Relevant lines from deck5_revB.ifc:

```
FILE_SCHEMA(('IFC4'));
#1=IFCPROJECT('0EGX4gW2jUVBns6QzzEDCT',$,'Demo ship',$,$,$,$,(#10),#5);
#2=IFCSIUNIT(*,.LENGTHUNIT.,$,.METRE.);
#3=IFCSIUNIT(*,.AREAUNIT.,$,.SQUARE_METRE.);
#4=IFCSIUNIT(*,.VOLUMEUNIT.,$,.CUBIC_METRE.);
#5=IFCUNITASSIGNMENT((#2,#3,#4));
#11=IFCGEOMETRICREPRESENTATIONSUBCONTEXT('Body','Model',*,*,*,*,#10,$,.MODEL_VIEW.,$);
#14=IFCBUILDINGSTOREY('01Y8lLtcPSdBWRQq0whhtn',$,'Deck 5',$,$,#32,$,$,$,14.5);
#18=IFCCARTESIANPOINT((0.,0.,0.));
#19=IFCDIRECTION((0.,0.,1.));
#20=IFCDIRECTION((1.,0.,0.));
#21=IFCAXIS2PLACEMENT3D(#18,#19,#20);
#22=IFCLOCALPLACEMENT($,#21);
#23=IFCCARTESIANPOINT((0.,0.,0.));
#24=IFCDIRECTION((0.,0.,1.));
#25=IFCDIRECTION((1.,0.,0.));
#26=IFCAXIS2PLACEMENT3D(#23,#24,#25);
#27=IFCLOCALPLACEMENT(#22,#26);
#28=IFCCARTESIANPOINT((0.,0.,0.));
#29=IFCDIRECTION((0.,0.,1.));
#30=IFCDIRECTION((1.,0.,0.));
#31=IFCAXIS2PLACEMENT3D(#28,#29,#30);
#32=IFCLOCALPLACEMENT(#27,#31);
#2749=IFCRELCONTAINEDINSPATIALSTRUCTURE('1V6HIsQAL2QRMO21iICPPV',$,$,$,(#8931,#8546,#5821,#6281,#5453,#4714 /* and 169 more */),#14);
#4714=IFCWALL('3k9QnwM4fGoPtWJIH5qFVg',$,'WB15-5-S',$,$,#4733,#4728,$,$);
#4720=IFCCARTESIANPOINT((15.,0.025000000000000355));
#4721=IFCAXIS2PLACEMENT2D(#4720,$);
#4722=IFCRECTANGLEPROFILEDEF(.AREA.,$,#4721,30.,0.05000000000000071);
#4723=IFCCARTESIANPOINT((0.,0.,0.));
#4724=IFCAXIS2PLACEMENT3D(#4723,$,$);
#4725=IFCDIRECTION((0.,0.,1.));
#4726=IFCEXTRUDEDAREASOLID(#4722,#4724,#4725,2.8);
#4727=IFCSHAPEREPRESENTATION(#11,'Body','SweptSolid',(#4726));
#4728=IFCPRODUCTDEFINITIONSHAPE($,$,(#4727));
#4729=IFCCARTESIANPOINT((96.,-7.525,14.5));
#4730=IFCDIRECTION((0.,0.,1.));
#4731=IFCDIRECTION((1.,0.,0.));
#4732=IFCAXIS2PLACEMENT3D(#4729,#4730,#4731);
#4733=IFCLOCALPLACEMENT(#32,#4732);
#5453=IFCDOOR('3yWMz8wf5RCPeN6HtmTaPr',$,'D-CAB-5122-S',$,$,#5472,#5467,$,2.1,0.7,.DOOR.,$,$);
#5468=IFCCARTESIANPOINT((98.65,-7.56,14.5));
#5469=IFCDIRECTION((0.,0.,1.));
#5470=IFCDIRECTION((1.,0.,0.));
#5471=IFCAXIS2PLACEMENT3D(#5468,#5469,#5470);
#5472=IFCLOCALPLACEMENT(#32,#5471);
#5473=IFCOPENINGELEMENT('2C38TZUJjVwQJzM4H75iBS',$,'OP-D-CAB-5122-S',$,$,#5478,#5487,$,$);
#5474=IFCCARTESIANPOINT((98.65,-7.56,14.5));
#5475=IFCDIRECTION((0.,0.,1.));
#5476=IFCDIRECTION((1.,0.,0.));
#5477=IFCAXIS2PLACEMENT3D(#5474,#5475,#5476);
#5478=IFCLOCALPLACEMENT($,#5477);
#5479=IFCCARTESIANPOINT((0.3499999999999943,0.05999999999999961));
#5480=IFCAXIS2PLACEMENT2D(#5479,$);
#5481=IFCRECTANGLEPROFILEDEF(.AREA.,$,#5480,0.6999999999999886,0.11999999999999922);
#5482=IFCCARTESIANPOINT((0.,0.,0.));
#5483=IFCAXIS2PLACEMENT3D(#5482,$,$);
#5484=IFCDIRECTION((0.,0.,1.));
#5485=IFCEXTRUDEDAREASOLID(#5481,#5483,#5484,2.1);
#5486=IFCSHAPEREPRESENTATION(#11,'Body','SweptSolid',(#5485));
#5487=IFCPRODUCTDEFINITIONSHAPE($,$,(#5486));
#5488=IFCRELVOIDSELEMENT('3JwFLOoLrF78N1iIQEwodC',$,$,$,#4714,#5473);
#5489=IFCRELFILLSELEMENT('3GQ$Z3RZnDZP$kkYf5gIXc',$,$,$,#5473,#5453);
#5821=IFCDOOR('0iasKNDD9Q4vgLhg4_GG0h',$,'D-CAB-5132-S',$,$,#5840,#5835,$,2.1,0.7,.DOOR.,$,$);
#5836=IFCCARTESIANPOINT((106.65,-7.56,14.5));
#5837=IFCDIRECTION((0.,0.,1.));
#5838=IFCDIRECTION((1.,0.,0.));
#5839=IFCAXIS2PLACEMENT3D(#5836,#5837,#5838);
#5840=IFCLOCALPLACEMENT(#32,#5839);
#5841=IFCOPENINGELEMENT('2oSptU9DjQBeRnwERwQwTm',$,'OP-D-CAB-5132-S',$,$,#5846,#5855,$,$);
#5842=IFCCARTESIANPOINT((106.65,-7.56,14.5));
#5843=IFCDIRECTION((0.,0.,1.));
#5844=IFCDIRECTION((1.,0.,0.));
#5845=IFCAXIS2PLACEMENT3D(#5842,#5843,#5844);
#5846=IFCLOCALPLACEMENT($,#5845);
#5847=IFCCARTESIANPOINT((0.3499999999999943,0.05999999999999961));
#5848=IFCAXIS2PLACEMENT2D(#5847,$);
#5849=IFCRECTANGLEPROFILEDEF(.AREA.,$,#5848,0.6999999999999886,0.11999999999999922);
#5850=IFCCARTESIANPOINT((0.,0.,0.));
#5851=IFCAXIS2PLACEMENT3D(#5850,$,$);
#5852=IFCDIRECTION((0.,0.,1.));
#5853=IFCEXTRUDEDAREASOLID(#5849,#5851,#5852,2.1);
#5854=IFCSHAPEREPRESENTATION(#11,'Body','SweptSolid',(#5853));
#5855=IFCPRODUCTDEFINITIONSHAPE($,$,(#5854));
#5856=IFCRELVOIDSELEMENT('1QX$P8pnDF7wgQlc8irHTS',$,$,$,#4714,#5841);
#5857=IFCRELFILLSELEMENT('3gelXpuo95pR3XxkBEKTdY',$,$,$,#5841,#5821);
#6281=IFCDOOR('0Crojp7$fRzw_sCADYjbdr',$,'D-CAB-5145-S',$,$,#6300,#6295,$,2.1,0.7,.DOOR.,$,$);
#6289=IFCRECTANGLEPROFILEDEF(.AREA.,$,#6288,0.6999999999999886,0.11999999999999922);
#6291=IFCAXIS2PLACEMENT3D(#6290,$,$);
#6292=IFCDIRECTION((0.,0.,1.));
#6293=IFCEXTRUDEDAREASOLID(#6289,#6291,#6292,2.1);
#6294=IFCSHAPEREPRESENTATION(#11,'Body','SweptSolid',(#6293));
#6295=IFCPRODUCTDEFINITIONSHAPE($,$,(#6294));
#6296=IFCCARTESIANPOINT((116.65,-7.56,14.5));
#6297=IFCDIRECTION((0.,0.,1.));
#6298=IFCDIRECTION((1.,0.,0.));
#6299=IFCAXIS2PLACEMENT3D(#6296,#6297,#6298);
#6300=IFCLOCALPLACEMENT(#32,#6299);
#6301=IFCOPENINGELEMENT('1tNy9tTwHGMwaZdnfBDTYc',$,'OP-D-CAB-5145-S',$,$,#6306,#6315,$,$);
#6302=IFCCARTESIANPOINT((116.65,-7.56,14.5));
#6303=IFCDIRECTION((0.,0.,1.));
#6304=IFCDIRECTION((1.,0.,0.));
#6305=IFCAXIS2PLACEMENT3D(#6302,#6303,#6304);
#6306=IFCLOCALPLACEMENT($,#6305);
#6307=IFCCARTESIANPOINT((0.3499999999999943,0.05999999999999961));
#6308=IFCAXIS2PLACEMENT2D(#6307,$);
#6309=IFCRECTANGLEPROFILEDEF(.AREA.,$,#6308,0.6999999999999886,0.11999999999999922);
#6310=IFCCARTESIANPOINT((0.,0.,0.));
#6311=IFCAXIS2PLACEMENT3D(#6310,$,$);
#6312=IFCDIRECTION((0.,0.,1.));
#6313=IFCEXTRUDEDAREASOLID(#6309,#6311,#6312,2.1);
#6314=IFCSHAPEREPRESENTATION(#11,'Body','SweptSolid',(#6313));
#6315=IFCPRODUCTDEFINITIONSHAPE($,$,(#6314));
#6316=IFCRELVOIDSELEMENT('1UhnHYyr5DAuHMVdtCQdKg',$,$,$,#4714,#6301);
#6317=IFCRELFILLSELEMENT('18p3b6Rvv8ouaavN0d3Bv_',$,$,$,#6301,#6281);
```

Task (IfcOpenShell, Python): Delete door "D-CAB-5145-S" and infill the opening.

```python
import ifcopenshell
import ifcopenshell.api.feature
import ifcopenshell.api.root
import ifcopenshell.geom
import ifcopenshell.util.shape

model = ifcopenshell.open("deck5_revB.ifc")
settings = ifcopenshell.geom.settings()


def volume(element):
    """Net volume in cubic metres, openings subtracted."""
    shape = ifcopenshell.geom.create_shape(settings, element)
    return ifcopenshell.util.shape.get_volume(shape.geometry)


door = model.by_guid("0Crojp7$fRzw_sCADYjbdr")
opening = door.FillsVoids[0].RelatingOpeningElement
wall = opening.VoidsElements[0].RelatingBuildingElement
before = volume(wall)

ifcopenshell.api.root.remove_product(model, product=door)
ifcopenshell.api.feature.remove_feature(model, feature=opening)

after = volume(wall)

print(f"wall volume {before:.3f} -> {after:.3f} m3")

model.write("deck5_revB-out.ifc")
```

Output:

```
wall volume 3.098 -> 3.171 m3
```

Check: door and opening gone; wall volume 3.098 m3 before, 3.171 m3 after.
